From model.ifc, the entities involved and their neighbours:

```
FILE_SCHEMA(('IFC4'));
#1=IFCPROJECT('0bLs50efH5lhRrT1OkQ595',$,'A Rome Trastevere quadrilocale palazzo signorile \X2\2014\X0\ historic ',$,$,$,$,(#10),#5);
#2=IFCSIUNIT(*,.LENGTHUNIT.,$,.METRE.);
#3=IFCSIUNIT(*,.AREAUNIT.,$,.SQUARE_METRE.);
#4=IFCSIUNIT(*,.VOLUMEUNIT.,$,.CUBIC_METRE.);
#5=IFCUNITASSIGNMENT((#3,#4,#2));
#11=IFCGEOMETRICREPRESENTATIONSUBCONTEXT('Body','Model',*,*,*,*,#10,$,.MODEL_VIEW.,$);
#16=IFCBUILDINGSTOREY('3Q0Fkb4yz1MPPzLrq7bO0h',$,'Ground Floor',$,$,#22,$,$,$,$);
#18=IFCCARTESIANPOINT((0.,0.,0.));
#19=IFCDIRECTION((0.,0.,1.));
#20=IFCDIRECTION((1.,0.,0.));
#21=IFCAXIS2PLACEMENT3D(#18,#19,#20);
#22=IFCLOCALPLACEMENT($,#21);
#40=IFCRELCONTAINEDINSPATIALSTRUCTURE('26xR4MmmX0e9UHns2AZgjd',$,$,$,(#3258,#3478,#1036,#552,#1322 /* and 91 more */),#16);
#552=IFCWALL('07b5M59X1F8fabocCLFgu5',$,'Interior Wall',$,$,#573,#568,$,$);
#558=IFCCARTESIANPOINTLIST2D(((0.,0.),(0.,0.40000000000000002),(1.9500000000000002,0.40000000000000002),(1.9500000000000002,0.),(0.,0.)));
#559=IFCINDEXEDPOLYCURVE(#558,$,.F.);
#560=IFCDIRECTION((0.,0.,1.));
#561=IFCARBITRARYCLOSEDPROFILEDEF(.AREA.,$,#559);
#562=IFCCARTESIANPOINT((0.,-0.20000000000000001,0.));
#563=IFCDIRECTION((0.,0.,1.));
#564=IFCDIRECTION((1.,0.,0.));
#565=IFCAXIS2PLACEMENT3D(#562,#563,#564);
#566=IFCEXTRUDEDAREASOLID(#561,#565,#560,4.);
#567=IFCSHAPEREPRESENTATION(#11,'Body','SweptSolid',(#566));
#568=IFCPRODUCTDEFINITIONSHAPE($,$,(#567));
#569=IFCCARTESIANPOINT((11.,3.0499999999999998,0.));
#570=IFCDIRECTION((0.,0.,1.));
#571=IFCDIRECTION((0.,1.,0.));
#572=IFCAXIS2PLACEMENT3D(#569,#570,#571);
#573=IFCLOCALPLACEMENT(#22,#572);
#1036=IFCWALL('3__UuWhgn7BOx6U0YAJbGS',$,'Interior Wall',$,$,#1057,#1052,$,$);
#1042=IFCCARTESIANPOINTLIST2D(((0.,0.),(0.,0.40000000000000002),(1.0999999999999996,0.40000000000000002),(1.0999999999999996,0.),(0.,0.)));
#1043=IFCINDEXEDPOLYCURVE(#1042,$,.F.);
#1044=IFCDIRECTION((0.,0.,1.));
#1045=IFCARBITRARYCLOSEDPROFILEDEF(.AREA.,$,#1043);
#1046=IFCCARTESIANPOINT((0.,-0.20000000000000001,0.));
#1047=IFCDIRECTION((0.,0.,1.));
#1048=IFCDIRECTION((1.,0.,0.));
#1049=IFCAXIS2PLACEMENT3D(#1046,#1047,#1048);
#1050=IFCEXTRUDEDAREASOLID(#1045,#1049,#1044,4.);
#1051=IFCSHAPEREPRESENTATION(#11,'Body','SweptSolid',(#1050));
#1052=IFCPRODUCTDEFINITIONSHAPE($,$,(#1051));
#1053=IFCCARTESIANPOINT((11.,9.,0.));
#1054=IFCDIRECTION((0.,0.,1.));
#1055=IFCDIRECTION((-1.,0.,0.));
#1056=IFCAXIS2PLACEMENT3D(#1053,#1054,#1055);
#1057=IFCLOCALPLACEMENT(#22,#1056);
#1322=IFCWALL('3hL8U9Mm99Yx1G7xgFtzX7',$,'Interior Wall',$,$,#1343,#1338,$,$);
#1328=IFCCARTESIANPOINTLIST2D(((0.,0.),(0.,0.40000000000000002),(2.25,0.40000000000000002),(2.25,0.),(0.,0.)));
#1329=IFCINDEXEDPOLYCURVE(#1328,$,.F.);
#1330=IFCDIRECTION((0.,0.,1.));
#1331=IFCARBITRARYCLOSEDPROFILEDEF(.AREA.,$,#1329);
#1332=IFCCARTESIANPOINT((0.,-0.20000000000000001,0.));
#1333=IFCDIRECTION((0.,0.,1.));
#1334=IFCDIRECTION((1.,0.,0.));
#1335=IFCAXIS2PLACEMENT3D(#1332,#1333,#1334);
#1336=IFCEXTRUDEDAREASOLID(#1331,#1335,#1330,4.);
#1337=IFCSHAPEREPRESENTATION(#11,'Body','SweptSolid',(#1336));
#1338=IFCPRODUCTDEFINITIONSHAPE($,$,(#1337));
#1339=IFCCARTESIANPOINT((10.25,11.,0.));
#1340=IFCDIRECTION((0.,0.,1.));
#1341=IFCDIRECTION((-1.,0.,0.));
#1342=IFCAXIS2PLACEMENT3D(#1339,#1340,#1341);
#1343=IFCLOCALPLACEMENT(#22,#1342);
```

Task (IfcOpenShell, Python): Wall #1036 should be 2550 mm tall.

```python
import ifcopenshell
import ifcopenshell.geom
import ifcopenshell.util.representation
import ifcopenshell.util.shape
import ifcopenshell.util.unit

model = ifcopenshell.open("model.ifc")
unit_scale = ifcopenshell.util.unit.calculate_unit_scale(model)
settings = ifcopenshell.geom.settings()


def volume(element):
    """Net volume in cubic metres, openings subtracted."""
    shape = ifcopenshell.geom.create_shape(settings, element)
    return ifcopenshell.util.shape.get_volume(shape.geometry)


wall = model.by_guid("3__UuWhgn7BOx6U0YAJbGS")
before = volume(wall)

body = ifcopenshell.util.representation.get_representation(wall, "Model", "Body")
solid = body.Items[0]
old_height = solid.Depth
solid.Depth = 2.55 / unit_scale
after = volume(wall)

print(f"height {old_height:g} -> {solid.Depth:g}, volume {before:.3f} -> {after:.3f} m3")

model.write("model_updated.ifc")
```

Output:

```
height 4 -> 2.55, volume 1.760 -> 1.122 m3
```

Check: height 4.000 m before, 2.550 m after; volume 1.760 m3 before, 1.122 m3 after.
